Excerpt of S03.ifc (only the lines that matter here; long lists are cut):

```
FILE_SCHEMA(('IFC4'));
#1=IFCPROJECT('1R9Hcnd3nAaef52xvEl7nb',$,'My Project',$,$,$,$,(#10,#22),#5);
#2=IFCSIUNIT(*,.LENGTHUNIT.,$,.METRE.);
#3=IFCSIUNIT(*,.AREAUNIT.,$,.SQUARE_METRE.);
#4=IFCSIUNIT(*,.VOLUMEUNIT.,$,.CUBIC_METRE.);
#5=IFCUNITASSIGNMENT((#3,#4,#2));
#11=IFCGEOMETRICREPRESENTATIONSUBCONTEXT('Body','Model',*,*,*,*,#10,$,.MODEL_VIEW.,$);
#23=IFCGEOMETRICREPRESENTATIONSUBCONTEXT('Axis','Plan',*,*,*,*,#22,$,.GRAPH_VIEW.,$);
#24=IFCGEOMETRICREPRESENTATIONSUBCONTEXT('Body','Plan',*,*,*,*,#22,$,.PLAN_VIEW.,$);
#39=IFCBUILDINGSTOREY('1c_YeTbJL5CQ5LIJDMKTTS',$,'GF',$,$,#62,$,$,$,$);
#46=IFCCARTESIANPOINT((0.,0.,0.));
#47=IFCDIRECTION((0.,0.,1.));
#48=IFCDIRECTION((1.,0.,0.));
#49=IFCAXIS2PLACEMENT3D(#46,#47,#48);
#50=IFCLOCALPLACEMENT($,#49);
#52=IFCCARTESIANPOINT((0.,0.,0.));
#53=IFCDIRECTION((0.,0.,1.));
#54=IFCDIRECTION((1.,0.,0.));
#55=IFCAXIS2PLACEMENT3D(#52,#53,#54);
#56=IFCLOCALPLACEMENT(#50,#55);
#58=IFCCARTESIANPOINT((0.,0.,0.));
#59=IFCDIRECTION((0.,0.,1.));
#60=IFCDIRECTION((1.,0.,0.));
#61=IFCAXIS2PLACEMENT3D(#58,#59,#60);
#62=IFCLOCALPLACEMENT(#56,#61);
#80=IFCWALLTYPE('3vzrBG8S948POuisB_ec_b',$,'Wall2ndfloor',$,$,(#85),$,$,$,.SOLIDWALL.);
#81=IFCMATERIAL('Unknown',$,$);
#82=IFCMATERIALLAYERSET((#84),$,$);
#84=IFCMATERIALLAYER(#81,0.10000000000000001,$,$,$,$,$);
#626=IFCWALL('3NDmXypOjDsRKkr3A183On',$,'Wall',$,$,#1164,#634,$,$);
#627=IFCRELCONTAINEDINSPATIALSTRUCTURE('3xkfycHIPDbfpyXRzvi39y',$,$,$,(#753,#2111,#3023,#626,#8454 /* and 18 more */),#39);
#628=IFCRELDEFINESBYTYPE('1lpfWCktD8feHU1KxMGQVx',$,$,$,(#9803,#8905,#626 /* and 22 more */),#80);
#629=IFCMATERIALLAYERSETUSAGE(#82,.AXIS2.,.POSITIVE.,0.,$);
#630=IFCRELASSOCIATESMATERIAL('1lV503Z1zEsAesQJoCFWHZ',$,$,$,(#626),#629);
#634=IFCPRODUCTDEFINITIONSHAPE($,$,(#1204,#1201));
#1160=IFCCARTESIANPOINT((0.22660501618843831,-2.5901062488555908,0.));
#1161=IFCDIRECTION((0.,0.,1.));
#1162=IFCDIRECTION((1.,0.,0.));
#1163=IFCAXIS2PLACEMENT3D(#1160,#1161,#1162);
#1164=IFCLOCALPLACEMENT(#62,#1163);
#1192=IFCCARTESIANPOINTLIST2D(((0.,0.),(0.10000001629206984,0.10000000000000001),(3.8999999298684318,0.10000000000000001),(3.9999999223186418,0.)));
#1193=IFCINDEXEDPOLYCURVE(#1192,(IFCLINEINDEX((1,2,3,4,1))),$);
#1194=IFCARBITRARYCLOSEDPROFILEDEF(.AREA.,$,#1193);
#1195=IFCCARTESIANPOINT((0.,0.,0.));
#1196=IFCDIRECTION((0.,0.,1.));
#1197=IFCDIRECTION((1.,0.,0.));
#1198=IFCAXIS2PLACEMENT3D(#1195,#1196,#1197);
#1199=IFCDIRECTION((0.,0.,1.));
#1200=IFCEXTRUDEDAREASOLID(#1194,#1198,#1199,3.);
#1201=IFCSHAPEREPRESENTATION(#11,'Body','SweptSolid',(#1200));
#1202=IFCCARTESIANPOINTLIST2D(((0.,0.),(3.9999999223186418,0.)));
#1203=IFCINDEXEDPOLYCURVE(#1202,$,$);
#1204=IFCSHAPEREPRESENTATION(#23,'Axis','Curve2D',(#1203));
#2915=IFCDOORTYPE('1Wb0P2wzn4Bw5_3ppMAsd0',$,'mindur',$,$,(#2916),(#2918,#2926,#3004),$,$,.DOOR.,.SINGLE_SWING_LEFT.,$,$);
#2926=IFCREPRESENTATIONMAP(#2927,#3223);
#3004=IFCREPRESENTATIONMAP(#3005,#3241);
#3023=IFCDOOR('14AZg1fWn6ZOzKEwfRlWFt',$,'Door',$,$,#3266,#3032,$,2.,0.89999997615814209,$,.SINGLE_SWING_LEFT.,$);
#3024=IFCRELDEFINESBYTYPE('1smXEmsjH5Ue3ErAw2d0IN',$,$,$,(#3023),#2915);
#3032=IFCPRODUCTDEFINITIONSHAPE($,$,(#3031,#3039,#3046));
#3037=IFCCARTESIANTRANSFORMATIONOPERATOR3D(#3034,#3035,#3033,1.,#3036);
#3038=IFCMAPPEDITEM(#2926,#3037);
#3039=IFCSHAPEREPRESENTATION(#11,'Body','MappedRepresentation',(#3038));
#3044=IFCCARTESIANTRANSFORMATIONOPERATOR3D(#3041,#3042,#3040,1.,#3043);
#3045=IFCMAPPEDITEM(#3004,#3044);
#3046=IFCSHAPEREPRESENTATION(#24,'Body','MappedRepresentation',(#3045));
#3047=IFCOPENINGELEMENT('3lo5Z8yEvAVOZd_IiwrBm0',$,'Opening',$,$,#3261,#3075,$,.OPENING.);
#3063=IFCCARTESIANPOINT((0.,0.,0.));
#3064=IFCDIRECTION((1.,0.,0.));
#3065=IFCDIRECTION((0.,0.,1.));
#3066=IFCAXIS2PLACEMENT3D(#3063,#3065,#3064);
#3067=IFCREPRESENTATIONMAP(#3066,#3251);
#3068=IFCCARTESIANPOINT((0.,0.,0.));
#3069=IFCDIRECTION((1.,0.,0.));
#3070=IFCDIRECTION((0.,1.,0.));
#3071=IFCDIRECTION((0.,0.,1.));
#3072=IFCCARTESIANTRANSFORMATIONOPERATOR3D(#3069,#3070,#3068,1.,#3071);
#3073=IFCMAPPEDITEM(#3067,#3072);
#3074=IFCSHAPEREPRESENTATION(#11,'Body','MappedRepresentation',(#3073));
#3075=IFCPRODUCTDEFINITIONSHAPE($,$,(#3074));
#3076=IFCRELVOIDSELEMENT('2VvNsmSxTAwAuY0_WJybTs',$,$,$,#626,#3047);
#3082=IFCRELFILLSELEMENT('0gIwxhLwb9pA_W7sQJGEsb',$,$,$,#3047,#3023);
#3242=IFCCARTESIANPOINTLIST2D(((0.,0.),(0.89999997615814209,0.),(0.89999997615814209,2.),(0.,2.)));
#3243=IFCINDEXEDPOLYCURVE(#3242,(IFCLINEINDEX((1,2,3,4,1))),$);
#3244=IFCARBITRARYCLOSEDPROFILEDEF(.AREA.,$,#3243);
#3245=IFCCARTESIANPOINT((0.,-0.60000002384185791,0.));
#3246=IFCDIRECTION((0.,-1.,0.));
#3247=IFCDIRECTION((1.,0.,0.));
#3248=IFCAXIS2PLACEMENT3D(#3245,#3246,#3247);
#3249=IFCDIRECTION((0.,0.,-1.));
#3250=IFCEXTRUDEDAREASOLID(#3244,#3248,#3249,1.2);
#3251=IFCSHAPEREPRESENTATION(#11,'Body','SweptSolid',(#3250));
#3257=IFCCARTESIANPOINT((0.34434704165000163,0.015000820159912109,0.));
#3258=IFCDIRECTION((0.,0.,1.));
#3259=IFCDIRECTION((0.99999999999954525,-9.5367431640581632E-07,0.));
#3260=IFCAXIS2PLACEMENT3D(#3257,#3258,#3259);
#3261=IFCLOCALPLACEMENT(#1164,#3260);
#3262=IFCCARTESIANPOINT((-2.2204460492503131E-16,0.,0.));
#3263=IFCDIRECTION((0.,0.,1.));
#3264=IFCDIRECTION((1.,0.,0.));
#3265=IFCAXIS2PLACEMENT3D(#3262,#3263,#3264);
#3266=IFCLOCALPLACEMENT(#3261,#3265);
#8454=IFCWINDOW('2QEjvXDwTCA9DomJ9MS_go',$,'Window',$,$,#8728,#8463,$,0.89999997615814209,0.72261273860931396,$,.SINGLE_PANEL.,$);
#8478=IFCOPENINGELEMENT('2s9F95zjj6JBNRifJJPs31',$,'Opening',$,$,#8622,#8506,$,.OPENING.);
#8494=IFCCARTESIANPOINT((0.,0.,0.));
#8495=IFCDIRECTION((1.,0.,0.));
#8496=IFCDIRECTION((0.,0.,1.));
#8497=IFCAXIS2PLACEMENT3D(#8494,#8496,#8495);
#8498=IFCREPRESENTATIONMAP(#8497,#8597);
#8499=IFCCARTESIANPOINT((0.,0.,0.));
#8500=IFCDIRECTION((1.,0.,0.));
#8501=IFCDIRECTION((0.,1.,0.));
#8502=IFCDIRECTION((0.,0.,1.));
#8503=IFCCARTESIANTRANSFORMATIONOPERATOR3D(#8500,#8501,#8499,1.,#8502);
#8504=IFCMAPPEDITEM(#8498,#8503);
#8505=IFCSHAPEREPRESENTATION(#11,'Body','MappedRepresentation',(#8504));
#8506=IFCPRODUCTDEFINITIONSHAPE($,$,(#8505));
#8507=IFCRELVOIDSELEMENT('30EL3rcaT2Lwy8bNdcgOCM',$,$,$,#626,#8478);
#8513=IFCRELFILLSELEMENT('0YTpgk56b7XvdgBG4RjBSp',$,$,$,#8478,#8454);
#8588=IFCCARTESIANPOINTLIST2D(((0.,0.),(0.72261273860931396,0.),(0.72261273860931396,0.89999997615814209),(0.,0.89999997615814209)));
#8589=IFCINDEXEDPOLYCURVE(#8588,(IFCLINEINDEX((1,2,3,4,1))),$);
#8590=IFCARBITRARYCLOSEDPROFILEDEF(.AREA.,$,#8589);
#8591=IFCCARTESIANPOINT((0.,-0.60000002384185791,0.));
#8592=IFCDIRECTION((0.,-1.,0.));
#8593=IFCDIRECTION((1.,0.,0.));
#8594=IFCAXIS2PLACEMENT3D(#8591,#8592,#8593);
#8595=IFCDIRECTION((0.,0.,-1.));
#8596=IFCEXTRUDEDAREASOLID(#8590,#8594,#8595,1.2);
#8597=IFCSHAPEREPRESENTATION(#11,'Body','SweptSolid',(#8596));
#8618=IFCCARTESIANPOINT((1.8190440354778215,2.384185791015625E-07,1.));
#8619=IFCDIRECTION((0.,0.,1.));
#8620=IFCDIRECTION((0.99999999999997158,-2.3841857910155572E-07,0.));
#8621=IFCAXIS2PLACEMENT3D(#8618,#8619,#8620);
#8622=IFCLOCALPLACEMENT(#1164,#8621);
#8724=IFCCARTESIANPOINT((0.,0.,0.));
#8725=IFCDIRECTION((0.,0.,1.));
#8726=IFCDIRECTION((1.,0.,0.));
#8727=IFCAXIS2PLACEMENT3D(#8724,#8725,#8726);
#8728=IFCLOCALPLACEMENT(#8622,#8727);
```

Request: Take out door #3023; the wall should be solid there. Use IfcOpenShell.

```python
import ifcopenshell
import ifcopenshell.api.feature
import ifcopenshell.api.root
import ifcopenshell.geom
import ifcopenshell.util.shape

model = ifcopenshell.open("S03.ifc")
settings = ifcopenshell.geom.settings()


def volume(element):
    """Net volume in cubic metres, openings subtracted."""
    shape = ifcopenshell.geom.create_shape(settings, element)
    return ifcopenshell.util.shape.get_volume(shape.geometry)


door = model.by_id(3023)
opening = door.FillsVoids[0].RelatingOpeningElement
wall = opening.VoidsElements[0].RelatingBuildingElement
before = volume(wall)

ifcopenshell.api.root.remove_product(model, product=door)
ifcopenshell.api.feature.remove_feature(model, feature=opening)

after = volume(wall)

print(f"wall volume {before:.3f} -> {after:.3f} m3")

model.write("S03-out.ifc")
```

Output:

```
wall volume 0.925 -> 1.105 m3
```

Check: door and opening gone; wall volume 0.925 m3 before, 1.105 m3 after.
